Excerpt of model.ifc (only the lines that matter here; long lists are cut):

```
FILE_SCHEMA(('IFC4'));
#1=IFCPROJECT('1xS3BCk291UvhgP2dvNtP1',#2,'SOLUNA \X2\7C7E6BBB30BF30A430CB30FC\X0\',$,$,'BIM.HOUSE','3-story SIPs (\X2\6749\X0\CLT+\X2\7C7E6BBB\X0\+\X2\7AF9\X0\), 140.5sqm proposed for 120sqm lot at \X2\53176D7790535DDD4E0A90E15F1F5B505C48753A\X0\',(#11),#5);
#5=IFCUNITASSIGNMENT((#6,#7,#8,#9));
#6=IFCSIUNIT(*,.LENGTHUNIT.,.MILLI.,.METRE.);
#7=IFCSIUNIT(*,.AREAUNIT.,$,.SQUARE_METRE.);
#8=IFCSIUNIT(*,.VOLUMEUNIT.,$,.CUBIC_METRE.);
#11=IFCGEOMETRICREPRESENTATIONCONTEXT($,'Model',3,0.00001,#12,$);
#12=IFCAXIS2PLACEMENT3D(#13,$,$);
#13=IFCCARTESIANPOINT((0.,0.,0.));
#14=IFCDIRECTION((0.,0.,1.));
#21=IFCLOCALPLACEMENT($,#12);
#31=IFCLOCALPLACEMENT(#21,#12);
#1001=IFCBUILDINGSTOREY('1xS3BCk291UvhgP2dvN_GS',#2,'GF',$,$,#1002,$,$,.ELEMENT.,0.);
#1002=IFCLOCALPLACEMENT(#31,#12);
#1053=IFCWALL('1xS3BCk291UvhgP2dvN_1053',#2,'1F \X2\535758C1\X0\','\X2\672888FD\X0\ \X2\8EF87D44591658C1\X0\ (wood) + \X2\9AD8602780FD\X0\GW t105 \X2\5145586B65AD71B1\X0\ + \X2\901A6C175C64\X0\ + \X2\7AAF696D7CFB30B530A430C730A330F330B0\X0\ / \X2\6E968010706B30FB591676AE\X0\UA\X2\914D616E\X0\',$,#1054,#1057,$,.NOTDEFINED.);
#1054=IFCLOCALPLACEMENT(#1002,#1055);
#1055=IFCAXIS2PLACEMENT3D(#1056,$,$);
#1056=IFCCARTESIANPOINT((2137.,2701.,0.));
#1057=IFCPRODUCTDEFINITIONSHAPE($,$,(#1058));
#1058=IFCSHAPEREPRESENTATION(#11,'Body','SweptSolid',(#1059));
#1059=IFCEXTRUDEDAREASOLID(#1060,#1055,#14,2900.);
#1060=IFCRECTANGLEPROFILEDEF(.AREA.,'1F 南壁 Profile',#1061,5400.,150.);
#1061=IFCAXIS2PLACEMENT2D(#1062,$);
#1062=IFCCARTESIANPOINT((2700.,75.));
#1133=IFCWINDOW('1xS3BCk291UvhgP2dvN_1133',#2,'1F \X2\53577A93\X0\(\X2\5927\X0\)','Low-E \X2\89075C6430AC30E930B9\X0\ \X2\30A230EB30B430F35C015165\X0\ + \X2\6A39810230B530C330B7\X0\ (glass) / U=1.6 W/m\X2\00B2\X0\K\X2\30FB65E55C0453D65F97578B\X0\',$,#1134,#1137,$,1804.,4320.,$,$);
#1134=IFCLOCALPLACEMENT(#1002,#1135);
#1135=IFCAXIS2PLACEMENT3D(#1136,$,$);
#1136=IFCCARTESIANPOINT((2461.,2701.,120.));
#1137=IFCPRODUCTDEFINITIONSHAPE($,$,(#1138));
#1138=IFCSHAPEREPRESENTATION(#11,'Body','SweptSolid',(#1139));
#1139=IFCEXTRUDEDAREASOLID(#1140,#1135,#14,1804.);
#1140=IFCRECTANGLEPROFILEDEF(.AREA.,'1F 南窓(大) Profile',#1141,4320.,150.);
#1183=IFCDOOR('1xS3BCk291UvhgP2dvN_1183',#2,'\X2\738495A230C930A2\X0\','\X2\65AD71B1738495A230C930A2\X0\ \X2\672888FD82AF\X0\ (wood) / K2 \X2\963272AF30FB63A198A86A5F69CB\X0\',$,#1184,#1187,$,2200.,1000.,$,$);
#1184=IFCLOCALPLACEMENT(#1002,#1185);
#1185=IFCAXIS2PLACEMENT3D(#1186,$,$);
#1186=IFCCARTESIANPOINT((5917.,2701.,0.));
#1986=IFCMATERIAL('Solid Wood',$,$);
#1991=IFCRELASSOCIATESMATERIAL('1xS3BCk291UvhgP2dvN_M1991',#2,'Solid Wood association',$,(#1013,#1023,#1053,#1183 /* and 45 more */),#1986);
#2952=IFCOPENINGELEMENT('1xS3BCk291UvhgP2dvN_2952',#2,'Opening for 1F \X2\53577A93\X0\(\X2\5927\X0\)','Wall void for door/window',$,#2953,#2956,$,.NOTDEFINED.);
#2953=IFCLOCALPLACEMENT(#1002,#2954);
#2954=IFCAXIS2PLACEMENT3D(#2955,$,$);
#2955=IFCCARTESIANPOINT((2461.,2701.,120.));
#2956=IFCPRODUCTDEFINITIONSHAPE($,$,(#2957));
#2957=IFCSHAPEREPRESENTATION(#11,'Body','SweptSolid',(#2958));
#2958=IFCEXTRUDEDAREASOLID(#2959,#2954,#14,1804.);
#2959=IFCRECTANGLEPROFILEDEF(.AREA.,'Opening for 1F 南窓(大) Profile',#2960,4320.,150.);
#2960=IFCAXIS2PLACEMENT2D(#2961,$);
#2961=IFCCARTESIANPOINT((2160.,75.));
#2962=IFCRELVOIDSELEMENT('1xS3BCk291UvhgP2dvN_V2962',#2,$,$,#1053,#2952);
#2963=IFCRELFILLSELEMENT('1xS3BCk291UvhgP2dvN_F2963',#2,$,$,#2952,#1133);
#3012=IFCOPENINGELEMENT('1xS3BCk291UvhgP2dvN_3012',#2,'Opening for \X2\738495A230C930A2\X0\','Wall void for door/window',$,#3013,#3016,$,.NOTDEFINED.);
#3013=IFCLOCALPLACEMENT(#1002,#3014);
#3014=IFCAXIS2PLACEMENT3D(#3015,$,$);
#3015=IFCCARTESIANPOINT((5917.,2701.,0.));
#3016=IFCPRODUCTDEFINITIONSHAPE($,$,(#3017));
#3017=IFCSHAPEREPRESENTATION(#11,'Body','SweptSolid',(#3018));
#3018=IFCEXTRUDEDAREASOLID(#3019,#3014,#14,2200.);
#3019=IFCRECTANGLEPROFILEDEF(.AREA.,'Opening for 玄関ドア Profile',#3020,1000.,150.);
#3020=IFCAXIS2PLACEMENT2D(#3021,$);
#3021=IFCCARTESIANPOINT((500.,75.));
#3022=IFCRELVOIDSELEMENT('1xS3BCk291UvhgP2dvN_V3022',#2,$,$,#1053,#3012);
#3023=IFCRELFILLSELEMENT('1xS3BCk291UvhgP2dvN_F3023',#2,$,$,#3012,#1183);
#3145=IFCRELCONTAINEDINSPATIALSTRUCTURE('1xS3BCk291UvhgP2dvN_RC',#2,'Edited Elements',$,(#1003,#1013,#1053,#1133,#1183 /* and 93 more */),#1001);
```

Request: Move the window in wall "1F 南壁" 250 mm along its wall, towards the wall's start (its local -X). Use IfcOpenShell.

```python
import ifcopenshell
import ifcopenshell.api.geometry
import ifcopenshell.util.placement

model = ifcopenshell.open("model.ifc")

window = model.by_id(1133)
opening = window.FillsVoids[0].RelatingOpeningElement
wall = opening.VoidsElements[0].RelatingBuildingElement

wall_matrix = ifcopenshell.util.placement.get_local_placement(wall.ObjectPlacement)
shift = wall_matrix[:3, 0] * -250.0
before = ifcopenshell.util.placement.get_local_placement(window.ObjectPlacement)[:3, 3].copy()

# The window is not placed relative to its opening, so move both.
for product in (opening, window):
    matrix = ifcopenshell.util.placement.get_local_placement(product.ObjectPlacement)
    matrix[:3, 3] += shift
    ifcopenshell.api.geometry.edit_object_placement(model, product=product, matrix=matrix, is_si=False)

after = ifcopenshell.util.placement.get_local_placement(window.ObjectPlacement)[:3, 3]
print("window moved by", (after - before).round(3) + 0.0)

model.write("model_updated.ifc")
```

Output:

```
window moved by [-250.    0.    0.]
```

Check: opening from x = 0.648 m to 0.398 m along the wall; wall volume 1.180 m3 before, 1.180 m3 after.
